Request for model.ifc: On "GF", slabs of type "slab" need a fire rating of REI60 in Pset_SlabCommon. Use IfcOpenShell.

First a look at what the model holds.

```python
import ifcopenshell
import ifcopenshell.util.element

model = ifcopenshell.open("model.ifc")
print(model.schema)
storey = next(s for s in model.by_type("IfcBuildingStorey") if s.Name == "GF")
slabs = [e for e in ifcopenshell.util.element.get_decomposition(storey) if e.is_a("IfcSlab")]
seen = {}
for e in slabs:
    element_type = ifcopenshell.util.element.get_type(e)
    key = (element_type.Name if element_type != e and element_type else None, ifcopenshell.util.element.get_pset(e, "Pset_SlabCommon", "FireRating"))
    seen[key] = seen.get(key, 0) + 1
for (name, value), count in sorted(seen.items(), key=str):
    print(count, "x", name, "|", value)
```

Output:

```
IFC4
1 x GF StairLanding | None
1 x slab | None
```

```python
import ifcopenshell
import ifcopenshell.api.pset
import ifcopenshell.util.element

model = ifcopenshell.open("model.ifc")

storey = next(s for s in model.by_type("IfcBuildingStorey") if s.Name == "GF")
slabs = [e for e in ifcopenshell.util.element.get_decomposition(storey) if e.is_a("IfcSlab")]

count = 0
for e in slabs:
    element_type = ifcopenshell.util.element.get_type(e)
    if element_type in (None, e) or element_type.Name != "slab":
        continue
    # add_pset returns the element's existing set when there is one.
    pset = ifcopenshell.api.pset.add_pset(model, product=e, name="Pset_SlabCommon")
    ifcopenshell.api.pset.edit_pset(model, pset=pset, properties={"FireRating": "REI60"})
    count += 1

print(count, "slabs updated")

model.write("model_updated.ifc")
```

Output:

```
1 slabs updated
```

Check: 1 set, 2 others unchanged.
